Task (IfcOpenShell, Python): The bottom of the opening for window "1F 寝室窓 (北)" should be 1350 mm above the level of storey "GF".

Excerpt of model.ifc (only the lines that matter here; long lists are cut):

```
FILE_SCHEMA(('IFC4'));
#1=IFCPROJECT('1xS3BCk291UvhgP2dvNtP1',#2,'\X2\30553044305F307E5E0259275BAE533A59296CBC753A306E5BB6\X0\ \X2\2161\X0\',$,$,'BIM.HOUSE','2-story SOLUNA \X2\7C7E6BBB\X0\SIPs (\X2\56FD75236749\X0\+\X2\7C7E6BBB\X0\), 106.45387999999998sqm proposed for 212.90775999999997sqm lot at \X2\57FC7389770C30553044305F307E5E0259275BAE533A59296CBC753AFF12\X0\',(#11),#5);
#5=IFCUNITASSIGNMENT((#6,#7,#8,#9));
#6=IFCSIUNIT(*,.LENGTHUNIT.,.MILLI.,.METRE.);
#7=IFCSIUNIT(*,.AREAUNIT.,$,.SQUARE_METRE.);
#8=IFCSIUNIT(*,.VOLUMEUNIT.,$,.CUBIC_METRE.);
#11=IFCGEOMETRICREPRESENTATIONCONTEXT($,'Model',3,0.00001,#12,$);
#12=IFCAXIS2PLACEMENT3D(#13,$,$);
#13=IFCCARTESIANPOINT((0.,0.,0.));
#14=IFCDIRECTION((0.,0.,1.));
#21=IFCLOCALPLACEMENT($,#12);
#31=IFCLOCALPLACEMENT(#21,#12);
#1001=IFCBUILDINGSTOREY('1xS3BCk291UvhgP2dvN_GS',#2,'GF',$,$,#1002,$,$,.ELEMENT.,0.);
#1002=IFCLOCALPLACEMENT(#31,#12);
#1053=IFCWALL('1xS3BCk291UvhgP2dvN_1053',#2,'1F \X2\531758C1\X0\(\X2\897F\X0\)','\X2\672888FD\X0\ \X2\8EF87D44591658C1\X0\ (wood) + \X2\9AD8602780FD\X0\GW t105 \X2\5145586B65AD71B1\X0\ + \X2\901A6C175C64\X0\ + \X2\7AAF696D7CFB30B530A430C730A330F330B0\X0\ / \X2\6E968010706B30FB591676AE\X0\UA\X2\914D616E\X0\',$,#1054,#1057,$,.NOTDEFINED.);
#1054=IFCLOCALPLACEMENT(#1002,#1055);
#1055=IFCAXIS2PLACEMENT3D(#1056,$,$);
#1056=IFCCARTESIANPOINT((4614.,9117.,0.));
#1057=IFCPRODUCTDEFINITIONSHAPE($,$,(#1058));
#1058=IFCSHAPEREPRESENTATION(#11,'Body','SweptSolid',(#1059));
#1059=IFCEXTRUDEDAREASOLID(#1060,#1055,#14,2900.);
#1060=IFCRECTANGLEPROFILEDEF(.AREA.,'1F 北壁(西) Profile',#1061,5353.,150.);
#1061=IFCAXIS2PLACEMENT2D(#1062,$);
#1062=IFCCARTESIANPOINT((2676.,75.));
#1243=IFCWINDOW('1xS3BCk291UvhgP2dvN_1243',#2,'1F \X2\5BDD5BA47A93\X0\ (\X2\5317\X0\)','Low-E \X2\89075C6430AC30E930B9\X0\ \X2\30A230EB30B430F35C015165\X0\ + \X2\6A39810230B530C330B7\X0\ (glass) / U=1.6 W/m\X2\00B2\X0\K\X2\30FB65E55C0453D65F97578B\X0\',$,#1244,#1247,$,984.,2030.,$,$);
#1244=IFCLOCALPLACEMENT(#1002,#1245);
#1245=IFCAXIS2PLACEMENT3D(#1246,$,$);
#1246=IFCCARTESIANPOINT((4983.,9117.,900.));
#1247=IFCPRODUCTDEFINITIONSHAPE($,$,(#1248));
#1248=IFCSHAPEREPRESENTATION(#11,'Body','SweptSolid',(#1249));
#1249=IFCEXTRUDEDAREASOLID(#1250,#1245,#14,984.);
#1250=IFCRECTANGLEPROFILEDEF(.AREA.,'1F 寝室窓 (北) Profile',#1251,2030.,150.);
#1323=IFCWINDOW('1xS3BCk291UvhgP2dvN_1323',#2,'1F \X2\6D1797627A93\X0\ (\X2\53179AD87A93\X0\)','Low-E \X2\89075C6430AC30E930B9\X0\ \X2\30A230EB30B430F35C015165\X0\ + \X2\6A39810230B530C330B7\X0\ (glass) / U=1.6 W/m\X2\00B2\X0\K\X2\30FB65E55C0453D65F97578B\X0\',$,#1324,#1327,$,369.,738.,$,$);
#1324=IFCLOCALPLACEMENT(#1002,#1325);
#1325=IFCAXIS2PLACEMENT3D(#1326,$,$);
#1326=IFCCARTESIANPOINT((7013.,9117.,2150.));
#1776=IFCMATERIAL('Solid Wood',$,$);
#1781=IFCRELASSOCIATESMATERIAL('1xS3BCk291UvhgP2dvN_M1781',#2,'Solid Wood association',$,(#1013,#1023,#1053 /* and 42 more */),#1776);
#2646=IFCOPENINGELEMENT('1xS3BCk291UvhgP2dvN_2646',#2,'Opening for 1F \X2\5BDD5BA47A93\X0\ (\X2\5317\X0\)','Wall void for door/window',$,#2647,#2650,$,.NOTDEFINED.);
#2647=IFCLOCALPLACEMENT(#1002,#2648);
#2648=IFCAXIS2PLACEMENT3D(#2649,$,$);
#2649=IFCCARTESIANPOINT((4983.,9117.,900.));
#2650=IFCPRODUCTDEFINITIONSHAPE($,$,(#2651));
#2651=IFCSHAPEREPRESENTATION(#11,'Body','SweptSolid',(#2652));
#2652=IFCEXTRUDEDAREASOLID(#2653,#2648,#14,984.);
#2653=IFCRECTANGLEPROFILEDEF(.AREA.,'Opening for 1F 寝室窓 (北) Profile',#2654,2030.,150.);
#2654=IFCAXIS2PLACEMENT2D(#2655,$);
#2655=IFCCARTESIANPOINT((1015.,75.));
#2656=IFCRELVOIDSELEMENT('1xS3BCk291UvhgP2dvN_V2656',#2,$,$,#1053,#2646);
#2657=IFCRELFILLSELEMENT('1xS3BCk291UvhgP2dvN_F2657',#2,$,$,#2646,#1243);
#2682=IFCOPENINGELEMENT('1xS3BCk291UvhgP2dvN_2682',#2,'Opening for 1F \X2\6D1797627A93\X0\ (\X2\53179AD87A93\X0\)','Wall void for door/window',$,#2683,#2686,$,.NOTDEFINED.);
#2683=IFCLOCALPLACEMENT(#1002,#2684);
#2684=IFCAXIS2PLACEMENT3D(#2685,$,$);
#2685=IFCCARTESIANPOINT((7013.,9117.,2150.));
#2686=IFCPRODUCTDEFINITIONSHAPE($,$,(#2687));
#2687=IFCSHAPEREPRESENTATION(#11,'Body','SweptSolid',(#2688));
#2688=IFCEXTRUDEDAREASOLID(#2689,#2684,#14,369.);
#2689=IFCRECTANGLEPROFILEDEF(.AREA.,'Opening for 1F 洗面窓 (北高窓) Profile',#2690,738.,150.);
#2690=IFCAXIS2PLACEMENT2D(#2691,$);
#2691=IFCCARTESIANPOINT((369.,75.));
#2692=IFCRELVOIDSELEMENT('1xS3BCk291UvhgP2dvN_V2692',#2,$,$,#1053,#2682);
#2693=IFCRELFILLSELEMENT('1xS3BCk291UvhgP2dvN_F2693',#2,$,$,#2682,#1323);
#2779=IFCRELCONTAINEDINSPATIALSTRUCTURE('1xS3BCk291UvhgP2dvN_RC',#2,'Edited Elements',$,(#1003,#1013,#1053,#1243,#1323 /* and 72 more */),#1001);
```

```python
import numpy as np
import ifcopenshell
import ifcopenshell.api.geometry
import ifcopenshell.geom
import ifcopenshell.util.element
import ifcopenshell.util.placement
import ifcopenshell.util.shape
import ifcopenshell.util.unit

model = ifcopenshell.open("model.ifc")
unit_scale = ifcopenshell.util.unit.calculate_unit_scale(model)

window = model.by_guid("1xS3BCk291UvhgP2dvN_1243")
opening = window.FillsVoids[0].RelatingOpeningElement
storey = ifcopenshell.util.element.get_container(window, ifc_class="IfcBuildingStorey")
level = ifcopenshell.util.placement.get_local_placement(storey.ObjectPlacement)[2, 3]

# The opening's origin need not be at the sill, so measure its lowest point.
shape = ifcopenshell.geom.create_shape(ifcopenshell.geom.settings(), opening)
bottom = ifcopenshell.util.shape.get_shape_bottom_elevation(shape, shape.geometry) / unit_scale
dz = level + 1.35 / unit_scale - bottom

shift = np.array([0.0, 0.0, dz])
# The window is not placed relative to its opening, so move both.
for product in (opening, window):
    matrix = ifcopenshell.util.placement.get_local_placement(product.ObjectPlacement)
    matrix[:3, 3] += shift
    ifcopenshell.api.geometry.edit_object_placement(model, product=product, matrix=matrix, is_si=False)

print(f"moved by {dz * unit_scale:+.3f} m")

model.write("model_edited.ifc")
```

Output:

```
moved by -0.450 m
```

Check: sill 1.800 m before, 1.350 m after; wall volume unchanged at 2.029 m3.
